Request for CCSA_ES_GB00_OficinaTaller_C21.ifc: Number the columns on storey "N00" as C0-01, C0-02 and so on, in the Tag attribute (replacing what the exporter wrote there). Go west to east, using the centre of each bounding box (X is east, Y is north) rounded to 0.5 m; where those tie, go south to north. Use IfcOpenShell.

First a look at what the model holds.

```python
import ifcopenshell
import ifcopenshell.util.element
import ifcopenshell.util.placement

model = ifcopenshell.open("CCSA_ES_GB00_OficinaTaller_C21.ifc")
print(model.schema)
storey = next(s for s in model.by_type("IfcBuildingStorey") if s.Name == "N00")
columns = [e for e in ifcopenshell.util.element.get_decomposition(storey) if e.is_a("IfcColumn")]
for e in sorted(columns, key=lambda e: e.id()):
    origin = ifcopenshell.util.placement.get_local_placement(e.ObjectPlacement)[:3, 3]
    print(e.id(), e.Tag, e.Name, origin.round(2) + 0.0, sep=" | ")
```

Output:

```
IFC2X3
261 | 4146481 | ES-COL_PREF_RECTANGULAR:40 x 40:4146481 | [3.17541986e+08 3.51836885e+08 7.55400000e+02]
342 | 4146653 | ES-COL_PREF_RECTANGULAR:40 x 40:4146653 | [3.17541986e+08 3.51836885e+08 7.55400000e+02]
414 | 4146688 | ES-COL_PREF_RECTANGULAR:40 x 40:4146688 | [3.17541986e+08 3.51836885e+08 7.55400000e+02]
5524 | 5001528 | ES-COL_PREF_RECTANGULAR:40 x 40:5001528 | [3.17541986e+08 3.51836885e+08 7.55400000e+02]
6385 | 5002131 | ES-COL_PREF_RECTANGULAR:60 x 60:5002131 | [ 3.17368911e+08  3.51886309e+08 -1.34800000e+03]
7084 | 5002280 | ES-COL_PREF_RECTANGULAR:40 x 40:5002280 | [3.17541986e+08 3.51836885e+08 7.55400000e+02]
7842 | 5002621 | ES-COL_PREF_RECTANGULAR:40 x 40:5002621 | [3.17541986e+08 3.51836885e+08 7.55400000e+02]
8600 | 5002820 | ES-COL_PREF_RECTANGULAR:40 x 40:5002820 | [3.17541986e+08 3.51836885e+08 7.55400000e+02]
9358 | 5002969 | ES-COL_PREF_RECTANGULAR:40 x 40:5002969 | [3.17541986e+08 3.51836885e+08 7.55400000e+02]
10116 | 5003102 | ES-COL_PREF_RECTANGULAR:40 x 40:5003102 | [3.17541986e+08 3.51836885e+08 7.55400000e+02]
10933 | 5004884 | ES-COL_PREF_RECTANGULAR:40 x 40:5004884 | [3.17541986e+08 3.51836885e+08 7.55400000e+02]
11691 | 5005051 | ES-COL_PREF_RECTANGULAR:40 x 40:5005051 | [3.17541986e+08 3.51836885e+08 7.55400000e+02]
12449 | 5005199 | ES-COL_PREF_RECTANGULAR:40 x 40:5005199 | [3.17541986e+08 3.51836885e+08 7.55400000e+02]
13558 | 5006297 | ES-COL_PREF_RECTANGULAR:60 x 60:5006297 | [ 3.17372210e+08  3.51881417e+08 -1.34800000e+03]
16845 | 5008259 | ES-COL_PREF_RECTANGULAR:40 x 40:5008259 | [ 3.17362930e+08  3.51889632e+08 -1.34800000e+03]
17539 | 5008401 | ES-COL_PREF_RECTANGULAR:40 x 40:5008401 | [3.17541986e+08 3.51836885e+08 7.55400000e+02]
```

```python
import ifcopenshell
import ifcopenshell.geom
import ifcopenshell.util.element
import ifcopenshell.util.shape

model = ifcopenshell.open("CCSA_ES_GB00_OficinaTaller_C21.ifc")
settings = ifcopenshell.geom.settings()
settings.set("use-world-coords", True)


def centre(element):
    shape = ifcopenshell.geom.create_shape(settings, element)
    return ifcopenshell.util.shape.get_bbox_centroid(shape.geometry)


storey = next(s for s in model.by_type("IfcBuildingStorey") if s.Name == "N00")
columns = [e for e in ifcopenshell.util.element.get_decomposition(storey) if e.is_a("IfcColumn")]

# Insertion points can sit at a corner or the storey origin, so sort by the geometry (in metres).
centres = {e: centre(e) for e in columns}
columns.sort(key=lambda e: (round(centres[e][0] / 0.5), centres[e][1]))

for i, e in enumerate(columns, start=1):
    number = f"C0-{i:02d}"
    e.Tag = number
    print(e.id(), number)

model.write("CCSA_ES_GB00_OficinaTaller_C21_edited.ifc")
```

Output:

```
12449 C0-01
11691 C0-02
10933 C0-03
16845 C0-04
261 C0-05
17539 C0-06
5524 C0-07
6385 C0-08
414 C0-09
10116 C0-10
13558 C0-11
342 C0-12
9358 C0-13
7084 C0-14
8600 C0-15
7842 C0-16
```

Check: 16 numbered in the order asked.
